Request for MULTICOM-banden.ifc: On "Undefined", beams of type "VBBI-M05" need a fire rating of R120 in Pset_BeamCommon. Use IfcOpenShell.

First a look at what the model holds.

```python
import ifcopenshell
import ifcopenshell.util.element

model = ifcopenshell.open("MULTICOM-banden.ifc")
print(model.schema)
storey = next(s for s in model.by_type("IfcBuildingStorey") if s.Name == "Undefined")
beams = [e for e in ifcopenshell.util.element.get_decomposition(storey) if e.is_a("IfcBeam")]
seen = {}
for e in beams:
    element_type = ifcopenshell.util.element.get_type(e)
    key = (element_type.Name if element_type != e and element_type else None, ifcopenshell.util.element.get_pset(e, "Pset_BeamCommon", "FireRating"))
    seen[key] = seen.get(key, 0) + 1
for (name, value), count in sorted(seen.items(), key=str):
    print(count, "x", name, "|", value)
```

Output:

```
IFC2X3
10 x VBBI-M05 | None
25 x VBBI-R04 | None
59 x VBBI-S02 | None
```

```python
import ifcopenshell
import ifcopenshell.api.pset
import ifcopenshell.util.element

model = ifcopenshell.open("MULTICOM-banden.ifc")

storey = next(s for s in model.by_type("IfcBuildingStorey") if s.Name == "Undefined")
beams = [e for e in ifcopenshell.util.element.get_decomposition(storey) if e.is_a("IfcBeam")]

count = 0
for e in beams:
    element_type = ifcopenshell.util.element.get_type(e)
    if element_type in (None, e) or element_type.Name != "VBBI-M05":
        continue
    # add_pset returns the element's existing set when there is one.
    pset = ifcopenshell.api.pset.add_pset(model, product=e, name="Pset_BeamCommon")
    ifcopenshell.api.pset.edit_pset(model, pset=pset, properties={"FireRating": "R120"})
    count += 1

print(count, "beams updated")

model.write("MULTICOM-banden_edited.ifc")
```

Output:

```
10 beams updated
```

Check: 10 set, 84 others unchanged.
